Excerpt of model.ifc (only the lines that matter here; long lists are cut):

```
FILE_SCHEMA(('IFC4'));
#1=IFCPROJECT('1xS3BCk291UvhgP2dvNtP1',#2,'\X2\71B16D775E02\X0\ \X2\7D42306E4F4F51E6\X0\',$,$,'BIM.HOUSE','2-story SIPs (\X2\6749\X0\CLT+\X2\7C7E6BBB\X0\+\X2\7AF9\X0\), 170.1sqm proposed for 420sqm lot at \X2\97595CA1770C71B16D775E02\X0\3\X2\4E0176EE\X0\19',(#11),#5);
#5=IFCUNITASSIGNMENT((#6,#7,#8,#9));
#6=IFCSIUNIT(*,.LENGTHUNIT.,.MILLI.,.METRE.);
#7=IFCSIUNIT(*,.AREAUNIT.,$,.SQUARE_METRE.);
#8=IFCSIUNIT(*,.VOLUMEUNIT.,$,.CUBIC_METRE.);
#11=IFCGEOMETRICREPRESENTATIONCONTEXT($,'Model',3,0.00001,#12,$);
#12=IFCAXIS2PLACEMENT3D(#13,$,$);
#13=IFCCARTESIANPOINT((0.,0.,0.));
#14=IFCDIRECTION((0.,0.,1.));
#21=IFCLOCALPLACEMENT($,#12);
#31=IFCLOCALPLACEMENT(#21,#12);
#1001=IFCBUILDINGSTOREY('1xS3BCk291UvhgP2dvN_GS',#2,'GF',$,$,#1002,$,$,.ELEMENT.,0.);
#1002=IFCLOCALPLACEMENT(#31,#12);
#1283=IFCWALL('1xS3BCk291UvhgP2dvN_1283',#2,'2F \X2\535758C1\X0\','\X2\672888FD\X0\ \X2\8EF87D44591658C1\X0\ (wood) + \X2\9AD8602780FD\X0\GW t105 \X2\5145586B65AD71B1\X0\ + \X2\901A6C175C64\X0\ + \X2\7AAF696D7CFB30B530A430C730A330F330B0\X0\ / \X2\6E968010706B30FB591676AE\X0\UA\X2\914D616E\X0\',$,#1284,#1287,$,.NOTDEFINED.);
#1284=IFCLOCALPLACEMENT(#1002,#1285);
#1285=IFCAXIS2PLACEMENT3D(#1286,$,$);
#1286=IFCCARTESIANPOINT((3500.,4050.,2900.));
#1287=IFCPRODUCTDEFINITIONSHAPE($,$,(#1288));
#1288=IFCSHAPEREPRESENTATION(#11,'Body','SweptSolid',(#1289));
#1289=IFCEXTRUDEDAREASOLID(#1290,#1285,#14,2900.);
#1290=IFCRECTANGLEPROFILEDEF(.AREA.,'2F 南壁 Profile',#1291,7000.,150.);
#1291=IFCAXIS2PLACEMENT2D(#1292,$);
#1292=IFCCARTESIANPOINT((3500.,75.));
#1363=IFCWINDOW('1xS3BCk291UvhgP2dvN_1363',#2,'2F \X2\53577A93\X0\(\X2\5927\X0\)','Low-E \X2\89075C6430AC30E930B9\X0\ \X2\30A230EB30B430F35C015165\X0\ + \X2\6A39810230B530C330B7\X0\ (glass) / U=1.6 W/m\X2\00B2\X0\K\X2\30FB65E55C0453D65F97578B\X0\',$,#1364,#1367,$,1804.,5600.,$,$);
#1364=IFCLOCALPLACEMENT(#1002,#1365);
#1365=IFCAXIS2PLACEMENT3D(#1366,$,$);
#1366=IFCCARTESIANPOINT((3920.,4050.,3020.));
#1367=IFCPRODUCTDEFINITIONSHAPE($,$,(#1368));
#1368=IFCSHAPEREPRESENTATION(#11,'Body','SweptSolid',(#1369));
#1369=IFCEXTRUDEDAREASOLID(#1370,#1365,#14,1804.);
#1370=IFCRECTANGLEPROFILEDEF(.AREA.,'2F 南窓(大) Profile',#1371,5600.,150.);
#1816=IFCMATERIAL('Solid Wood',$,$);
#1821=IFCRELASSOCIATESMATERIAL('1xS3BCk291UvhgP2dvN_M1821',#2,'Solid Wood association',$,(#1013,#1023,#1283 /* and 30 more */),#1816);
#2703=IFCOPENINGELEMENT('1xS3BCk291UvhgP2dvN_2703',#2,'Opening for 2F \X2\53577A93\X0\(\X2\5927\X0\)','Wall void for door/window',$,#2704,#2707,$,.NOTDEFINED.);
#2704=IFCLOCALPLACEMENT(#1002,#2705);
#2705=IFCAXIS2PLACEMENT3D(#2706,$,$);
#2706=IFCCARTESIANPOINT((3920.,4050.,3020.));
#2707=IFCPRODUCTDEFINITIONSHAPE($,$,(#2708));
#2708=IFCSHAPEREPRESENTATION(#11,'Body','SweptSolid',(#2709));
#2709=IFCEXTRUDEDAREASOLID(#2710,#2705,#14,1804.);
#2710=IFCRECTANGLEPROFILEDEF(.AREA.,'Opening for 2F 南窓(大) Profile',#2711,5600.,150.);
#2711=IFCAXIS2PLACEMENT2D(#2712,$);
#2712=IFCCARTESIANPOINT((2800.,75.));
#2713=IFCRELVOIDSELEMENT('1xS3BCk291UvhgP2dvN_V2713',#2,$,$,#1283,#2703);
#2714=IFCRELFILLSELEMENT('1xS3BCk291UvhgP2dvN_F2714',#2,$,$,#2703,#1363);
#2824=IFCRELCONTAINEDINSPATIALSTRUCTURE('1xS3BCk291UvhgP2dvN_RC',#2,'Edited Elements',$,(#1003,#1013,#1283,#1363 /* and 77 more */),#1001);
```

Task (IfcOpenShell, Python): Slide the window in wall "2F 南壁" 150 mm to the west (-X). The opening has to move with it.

```python
import ifcopenshell
import ifcopenshell.api.geometry
import ifcopenshell.util.placement
import ifcopenshell.util.unit

model = ifcopenshell.open("model.ifc")
unit_scale = ifcopenshell.util.unit.calculate_unit_scale(model)

window = model.by_guid("1xS3BCk291UvhgP2dvN_1363")
opening = window.FillsVoids[0].RelatingOpeningElement
wall = opening.VoidsElements[0].RelatingBuildingElement

wall_matrix = ifcopenshell.util.placement.get_local_placement(wall.ObjectPlacement)
shift = wall_matrix[:3, 0] * -0.15 / unit_scale
before = ifcopenshell.util.placement.get_local_placement(window.ObjectPlacement)[:3, 3].copy()

# The window is not placed relative to its opening, so move both.
for product in (opening, window):
    matrix = ifcopenshell.util.placement.get_local_placement(product.ObjectPlacement)
    matrix[:3, 3] += shift
    ifcopenshell.api.geometry.edit_object_placement(model, product=product, matrix=matrix, is_si=False)

after = ifcopenshell.util.placement.get_local_placement(window.ObjectPlacement)[:3, 3]
print("window moved by", (after - before).round(3) + 0.0)

model.write("model_v2.ifc")
```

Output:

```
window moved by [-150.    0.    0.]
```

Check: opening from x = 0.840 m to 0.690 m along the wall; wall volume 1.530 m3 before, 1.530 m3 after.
